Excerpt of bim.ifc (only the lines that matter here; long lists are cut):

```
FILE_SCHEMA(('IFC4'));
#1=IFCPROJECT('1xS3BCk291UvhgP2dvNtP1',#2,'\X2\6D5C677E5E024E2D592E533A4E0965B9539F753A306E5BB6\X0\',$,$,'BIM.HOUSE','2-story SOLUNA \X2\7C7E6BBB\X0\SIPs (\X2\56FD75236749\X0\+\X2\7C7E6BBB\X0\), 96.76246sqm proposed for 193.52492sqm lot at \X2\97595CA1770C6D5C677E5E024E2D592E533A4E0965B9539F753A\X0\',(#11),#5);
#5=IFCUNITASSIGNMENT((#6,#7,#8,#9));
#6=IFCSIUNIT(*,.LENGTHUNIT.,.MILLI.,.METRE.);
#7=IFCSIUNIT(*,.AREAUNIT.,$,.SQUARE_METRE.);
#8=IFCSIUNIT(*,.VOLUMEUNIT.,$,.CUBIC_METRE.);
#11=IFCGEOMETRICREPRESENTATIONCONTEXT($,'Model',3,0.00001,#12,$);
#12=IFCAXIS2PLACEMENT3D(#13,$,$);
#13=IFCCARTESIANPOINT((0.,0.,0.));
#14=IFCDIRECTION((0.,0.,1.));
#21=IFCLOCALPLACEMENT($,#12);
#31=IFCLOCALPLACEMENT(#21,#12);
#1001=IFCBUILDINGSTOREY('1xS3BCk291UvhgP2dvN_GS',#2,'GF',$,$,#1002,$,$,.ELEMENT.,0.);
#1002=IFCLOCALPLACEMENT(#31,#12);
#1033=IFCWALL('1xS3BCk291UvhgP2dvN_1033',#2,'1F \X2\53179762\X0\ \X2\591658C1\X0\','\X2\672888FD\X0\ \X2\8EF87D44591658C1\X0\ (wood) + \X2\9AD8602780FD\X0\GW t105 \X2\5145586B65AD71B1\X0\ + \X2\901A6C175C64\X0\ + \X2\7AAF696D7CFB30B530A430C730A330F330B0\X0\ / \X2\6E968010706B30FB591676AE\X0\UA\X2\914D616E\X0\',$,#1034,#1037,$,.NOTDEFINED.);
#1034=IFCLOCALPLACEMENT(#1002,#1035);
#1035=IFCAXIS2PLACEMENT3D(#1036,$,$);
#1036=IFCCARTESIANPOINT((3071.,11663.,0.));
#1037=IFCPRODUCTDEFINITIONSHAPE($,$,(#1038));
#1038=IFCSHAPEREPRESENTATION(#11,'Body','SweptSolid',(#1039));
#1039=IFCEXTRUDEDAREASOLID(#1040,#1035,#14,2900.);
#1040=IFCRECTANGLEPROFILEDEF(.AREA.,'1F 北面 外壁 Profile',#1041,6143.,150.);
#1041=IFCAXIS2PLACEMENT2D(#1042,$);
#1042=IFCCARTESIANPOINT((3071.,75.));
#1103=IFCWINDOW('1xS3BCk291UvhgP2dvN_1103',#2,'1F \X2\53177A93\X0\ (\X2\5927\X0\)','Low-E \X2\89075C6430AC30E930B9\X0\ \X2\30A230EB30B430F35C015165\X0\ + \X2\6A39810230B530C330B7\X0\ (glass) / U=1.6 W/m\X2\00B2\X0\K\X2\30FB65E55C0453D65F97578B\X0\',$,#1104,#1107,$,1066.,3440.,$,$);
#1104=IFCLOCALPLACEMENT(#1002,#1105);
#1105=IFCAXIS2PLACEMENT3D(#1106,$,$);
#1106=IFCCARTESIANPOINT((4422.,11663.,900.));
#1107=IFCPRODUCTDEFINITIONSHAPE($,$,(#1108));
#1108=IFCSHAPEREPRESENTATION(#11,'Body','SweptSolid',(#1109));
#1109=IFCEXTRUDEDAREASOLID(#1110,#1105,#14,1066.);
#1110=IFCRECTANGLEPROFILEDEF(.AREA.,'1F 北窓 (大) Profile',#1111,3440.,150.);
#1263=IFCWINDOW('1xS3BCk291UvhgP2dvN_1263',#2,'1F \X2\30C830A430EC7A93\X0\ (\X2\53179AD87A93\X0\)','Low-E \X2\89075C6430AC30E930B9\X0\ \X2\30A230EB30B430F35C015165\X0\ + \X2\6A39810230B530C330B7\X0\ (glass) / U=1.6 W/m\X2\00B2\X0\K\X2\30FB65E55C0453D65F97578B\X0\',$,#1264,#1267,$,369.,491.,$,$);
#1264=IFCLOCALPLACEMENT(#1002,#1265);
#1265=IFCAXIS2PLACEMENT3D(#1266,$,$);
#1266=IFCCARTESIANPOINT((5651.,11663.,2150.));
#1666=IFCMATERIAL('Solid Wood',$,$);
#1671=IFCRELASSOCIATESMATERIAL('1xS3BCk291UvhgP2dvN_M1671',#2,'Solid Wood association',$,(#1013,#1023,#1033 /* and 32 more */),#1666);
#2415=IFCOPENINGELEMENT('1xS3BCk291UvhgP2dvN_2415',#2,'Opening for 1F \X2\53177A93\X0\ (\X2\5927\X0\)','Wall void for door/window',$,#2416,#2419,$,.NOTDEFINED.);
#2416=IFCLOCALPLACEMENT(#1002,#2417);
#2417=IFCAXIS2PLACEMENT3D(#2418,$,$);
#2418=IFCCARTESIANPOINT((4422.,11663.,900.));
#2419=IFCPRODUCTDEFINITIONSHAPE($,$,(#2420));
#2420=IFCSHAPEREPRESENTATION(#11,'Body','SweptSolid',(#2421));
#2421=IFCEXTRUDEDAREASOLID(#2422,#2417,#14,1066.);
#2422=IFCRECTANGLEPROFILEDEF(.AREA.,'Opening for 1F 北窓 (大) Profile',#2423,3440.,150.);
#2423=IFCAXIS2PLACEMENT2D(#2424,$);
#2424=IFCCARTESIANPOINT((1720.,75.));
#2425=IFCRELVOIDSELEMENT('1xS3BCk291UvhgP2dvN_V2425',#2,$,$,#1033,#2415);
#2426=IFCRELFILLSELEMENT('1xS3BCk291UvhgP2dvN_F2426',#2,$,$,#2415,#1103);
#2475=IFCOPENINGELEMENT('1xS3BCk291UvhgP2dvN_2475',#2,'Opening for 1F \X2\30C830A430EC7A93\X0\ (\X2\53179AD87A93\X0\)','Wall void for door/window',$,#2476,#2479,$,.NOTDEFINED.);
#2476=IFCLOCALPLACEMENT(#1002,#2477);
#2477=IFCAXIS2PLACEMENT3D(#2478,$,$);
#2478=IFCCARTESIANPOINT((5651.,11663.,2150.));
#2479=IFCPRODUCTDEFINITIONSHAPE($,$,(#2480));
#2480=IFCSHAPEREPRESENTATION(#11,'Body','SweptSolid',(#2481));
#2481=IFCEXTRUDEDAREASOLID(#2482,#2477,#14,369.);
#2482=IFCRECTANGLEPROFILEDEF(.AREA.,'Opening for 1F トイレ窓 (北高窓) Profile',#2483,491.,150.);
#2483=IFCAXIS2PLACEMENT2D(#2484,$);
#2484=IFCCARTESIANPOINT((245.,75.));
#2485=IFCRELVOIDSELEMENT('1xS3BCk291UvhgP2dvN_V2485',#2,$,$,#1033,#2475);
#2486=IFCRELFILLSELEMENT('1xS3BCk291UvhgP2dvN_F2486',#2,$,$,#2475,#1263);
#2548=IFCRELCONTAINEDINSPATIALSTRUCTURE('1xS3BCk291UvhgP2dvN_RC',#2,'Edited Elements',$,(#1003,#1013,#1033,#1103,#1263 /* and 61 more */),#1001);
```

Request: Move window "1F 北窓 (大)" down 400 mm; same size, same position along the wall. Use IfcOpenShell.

```python
import numpy as np
import ifcopenshell
import ifcopenshell.api.geometry
import ifcopenshell.util.placement
import ifcopenshell.util.unit

model = ifcopenshell.open("bim.ifc")
unit_scale = ifcopenshell.util.unit.calculate_unit_scale(model)

window = model.by_id(1103)
opening = window.FillsVoids[0].RelatingOpeningElement
dz = -400.0

shift = np.array([0.0, 0.0, dz])
# The window is not placed relative to its opening, so move both.
for product in (opening, window):
    matrix = ifcopenshell.util.placement.get_local_placement(product.ObjectPlacement)
    matrix[:3, 3] += shift
    ifcopenshell.api.geometry.edit_object_placement(model, product=product, matrix=matrix, is_si=False)

print(f"moved by {dz * unit_scale:+.3f} m")

model.write("bim_edited.ifc")
```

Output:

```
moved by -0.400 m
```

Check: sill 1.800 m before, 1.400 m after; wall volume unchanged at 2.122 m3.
